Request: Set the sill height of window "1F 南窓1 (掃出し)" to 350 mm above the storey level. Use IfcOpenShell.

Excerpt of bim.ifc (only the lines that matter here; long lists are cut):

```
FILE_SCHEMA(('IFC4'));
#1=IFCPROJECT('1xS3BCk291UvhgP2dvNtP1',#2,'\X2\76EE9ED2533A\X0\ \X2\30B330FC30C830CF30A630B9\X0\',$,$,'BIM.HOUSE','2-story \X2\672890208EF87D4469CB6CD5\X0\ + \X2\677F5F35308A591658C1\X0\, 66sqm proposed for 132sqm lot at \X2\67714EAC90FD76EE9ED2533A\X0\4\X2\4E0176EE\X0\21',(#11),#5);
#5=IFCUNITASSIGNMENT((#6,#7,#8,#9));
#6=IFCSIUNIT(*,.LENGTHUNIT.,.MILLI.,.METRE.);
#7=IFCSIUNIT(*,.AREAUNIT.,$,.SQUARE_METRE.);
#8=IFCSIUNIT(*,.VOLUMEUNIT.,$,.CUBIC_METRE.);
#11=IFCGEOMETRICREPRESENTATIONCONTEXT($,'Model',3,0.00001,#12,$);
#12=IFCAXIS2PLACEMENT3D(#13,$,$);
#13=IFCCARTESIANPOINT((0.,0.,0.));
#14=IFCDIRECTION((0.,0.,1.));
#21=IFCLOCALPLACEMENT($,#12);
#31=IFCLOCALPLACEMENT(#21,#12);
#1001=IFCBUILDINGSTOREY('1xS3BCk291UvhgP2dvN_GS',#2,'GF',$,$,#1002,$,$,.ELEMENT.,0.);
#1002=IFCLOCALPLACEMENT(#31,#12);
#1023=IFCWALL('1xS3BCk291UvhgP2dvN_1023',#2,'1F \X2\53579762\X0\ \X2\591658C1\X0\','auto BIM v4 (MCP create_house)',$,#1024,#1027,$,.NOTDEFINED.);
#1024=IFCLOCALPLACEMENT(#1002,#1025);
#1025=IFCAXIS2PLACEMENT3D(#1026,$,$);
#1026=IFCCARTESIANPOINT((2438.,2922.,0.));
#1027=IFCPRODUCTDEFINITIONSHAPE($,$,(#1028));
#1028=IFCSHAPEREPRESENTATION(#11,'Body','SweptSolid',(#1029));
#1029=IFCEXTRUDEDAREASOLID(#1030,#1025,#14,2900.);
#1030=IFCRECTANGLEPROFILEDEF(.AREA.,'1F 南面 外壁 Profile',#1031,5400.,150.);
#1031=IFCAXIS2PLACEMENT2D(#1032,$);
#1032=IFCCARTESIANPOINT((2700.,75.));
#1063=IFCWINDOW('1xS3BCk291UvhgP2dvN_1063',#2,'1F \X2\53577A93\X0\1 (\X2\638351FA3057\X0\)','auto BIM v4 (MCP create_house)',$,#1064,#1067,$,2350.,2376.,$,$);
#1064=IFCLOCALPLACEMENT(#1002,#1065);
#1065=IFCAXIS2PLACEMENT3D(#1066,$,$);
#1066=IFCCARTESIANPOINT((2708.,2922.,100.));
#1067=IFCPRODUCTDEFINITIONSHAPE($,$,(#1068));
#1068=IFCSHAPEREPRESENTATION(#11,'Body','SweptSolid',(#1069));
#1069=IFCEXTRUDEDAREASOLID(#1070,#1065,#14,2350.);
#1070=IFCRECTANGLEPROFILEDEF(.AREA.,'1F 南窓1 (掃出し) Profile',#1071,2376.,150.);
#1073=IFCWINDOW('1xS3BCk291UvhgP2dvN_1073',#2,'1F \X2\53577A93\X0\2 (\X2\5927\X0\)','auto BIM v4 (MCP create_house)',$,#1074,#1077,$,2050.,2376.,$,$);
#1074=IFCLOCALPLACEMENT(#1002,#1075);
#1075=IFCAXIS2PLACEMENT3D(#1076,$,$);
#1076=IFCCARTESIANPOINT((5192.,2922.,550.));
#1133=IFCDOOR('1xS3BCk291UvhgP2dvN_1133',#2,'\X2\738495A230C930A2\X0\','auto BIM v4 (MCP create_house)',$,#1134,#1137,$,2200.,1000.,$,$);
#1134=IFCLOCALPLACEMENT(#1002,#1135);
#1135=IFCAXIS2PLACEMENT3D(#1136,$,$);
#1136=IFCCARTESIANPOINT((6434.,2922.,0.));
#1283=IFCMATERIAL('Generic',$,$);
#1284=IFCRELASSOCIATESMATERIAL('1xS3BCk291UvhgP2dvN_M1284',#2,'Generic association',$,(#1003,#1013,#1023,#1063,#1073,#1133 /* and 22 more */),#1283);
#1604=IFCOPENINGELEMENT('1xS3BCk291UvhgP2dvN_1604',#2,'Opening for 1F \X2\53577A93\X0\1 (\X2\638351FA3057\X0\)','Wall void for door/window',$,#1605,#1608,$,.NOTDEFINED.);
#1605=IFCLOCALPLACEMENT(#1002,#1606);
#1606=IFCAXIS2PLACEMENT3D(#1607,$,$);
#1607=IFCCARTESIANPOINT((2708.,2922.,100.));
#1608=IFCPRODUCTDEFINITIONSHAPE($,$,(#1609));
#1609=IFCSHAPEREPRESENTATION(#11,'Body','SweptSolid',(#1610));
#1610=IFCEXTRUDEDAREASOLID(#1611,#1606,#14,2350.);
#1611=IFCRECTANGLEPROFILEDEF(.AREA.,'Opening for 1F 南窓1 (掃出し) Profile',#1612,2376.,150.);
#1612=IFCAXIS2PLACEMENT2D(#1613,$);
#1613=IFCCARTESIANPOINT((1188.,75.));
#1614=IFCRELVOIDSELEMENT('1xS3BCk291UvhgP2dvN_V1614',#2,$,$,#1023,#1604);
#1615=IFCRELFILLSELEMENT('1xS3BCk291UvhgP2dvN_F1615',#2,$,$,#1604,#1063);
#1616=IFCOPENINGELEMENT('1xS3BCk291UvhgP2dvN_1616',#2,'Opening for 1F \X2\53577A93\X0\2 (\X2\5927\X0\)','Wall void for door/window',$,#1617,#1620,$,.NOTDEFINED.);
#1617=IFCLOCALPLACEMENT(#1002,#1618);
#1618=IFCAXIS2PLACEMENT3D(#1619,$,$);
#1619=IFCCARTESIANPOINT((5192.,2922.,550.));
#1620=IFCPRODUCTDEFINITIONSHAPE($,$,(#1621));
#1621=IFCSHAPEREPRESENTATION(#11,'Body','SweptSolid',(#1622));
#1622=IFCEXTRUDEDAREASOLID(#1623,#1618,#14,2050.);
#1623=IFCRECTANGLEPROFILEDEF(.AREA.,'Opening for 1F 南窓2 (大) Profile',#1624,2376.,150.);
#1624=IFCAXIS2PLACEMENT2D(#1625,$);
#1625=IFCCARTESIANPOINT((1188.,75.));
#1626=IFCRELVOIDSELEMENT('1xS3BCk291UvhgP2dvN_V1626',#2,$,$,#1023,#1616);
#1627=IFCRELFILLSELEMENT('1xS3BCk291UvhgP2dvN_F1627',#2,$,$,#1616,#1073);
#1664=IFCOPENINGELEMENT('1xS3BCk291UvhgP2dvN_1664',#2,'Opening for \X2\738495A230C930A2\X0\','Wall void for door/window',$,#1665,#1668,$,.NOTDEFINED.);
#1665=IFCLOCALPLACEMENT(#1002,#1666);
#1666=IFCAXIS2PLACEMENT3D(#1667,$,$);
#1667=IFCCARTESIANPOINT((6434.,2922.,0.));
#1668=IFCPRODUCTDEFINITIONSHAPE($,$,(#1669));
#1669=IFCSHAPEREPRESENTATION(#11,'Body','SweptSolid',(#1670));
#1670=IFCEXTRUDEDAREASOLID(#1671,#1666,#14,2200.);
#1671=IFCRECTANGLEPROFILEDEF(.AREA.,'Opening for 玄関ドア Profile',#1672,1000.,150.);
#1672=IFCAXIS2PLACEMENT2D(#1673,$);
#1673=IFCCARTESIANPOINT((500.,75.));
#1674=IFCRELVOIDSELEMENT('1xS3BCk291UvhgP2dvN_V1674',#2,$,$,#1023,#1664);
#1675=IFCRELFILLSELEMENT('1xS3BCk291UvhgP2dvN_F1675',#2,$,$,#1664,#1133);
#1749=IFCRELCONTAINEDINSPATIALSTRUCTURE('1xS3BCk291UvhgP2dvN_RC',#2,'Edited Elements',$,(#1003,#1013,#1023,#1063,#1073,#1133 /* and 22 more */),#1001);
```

```python
import numpy as np
import ifcopenshell
import ifcopenshell.api.geometry
import ifcopenshell.geom
import ifcopenshell.util.element
import ifcopenshell.util.placement
import ifcopenshell.util.shape
import ifcopenshell.util.unit

model = ifcopenshell.open("bim.ifc")
unit_scale = ifcopenshell.util.unit.calculate_unit_scale(model)

window = model.by_id(1063)
opening = window.FillsVoids[0].RelatingOpeningElement
storey = ifcopenshell.util.element.get_container(window, ifc_class="IfcBuildingStorey")
level = ifcopenshell.util.placement.get_local_placement(storey.ObjectPlacement)[2, 3]

# The opening's origin need not be at the sill, so measure its lowest point.
shape = ifcopenshell.geom.create_shape(ifcopenshell.geom.settings(), opening)
bottom = ifcopenshell.util.shape.get_shape_bottom_elevation(shape, shape.geometry) / unit_scale
dz = level + 0.35 / unit_scale - bottom

shift = np.array([0.0, 0.0, dz])
# The window is not placed relative to its opening, so move both.
for product in (opening, window):
    matrix = ifcopenshell.util.placement.get_local_placement(product.ObjectPlacement)
    matrix[:3, 3] += shift
    ifcopenshell.api.geometry.edit_object_placement(model, product=product, matrix=matrix, is_si=False)

print(f"moved by {dz * unit_scale:+.3f} m")

model.write("bim_updated.ifc")
```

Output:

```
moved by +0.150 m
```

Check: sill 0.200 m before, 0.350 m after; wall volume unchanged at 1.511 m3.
